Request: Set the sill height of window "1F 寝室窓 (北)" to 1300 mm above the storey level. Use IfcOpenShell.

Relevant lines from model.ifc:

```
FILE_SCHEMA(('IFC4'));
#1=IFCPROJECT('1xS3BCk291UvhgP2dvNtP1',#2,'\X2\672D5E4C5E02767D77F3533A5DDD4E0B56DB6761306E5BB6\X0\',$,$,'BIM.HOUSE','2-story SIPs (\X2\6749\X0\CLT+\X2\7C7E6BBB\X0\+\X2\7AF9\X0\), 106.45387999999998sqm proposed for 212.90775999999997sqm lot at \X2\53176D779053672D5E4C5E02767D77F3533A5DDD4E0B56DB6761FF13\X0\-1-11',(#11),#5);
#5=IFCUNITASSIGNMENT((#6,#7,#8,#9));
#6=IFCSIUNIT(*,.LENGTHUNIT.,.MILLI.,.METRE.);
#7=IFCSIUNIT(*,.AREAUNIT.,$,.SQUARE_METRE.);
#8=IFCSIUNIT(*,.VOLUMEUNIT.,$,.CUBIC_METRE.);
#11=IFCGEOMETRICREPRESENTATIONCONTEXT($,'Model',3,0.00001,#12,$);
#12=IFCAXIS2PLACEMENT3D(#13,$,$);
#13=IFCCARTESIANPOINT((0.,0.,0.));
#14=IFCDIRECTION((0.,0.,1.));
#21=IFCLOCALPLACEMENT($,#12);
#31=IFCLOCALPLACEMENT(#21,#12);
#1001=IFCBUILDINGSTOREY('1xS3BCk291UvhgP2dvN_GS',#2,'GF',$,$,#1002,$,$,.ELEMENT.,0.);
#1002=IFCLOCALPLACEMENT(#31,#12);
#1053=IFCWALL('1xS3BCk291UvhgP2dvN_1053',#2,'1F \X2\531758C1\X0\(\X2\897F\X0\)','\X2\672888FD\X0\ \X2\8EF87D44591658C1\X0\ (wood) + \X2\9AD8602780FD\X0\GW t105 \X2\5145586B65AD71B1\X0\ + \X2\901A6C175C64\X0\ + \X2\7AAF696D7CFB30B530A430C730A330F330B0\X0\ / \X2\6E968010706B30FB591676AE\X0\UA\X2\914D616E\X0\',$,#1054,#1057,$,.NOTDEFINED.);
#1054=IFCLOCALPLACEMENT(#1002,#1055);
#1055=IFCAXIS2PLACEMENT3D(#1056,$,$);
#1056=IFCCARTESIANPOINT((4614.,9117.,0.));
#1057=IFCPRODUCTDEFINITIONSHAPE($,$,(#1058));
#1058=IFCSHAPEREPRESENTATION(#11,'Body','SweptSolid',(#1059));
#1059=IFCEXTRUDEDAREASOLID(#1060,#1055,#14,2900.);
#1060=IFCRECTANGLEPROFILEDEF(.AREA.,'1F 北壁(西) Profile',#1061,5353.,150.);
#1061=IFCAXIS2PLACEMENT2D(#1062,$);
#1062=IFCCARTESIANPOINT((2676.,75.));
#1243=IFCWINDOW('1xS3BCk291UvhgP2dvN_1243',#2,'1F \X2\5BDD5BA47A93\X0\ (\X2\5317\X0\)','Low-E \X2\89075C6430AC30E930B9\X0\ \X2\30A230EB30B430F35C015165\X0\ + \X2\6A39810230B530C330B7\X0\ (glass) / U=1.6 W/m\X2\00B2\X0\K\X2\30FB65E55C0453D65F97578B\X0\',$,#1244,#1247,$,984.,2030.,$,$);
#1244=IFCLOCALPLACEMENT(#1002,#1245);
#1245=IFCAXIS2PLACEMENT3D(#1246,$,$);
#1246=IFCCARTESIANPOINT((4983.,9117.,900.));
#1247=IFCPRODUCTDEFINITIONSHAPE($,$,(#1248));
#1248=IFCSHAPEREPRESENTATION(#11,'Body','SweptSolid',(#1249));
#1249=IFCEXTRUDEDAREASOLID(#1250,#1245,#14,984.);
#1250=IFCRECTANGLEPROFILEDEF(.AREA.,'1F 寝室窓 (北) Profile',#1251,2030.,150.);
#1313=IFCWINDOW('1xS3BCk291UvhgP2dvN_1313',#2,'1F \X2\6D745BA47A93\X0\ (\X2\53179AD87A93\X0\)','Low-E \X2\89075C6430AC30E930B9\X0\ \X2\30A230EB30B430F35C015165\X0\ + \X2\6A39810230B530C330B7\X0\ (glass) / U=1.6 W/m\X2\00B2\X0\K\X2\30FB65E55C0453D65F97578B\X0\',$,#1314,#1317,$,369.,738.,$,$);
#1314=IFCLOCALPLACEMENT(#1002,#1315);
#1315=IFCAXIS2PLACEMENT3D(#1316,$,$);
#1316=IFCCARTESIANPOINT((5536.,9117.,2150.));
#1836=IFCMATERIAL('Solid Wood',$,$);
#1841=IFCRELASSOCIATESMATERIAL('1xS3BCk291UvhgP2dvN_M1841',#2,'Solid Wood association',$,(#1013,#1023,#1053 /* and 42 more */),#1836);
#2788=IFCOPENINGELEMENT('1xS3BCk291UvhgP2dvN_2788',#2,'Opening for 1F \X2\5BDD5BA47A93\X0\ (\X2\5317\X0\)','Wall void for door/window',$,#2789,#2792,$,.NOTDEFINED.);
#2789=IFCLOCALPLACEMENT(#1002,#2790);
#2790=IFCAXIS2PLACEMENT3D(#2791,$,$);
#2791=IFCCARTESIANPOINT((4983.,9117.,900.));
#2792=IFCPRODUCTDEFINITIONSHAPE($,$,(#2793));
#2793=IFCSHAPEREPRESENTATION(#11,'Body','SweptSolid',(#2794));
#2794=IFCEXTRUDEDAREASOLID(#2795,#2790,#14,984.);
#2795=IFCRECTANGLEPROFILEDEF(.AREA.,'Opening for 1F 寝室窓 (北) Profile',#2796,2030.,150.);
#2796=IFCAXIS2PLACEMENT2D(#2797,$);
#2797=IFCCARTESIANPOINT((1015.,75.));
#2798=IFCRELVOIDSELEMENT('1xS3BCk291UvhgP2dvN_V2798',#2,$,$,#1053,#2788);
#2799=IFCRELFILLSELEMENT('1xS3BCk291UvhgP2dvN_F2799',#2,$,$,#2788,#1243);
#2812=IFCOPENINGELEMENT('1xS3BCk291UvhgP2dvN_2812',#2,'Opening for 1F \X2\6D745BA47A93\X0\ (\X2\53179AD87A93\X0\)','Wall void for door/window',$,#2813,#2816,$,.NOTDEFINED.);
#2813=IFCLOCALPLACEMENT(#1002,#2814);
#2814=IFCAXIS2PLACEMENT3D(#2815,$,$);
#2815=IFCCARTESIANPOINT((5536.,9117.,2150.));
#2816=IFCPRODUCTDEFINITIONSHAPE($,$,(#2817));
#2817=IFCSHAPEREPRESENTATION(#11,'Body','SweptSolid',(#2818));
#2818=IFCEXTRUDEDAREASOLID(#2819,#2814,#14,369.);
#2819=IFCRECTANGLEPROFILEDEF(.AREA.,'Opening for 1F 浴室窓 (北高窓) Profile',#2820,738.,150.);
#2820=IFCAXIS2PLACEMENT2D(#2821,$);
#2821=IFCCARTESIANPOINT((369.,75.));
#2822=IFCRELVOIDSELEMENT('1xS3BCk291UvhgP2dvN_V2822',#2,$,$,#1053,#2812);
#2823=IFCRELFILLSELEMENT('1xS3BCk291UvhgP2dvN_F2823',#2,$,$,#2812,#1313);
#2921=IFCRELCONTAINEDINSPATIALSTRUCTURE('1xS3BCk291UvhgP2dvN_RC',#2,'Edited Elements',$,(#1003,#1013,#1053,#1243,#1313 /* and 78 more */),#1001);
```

```python
import numpy as np
import ifcopenshell
import ifcopenshell.api.geometry
import ifcopenshell.geom
import ifcopenshell.util.element
import ifcopenshell.util.placement
import ifcopenshell.util.shape
import ifcopenshell.util.unit

model = ifcopenshell.open("model.ifc")
unit_scale = ifcopenshell.util.unit.calculate_unit_scale(model)

window = model.by_guid("1xS3BCk291UvhgP2dvN_1243")
opening = window.FillsVoids[0].RelatingOpeningElement
storey = ifcopenshell.util.element.get_container(window, ifc_class="IfcBuildingStorey")
level = ifcopenshell.util.placement.get_local_placement(storey.ObjectPlacement)[2, 3]

# The opening's origin need not be at the sill, so measure its lowest point.
shape = ifcopenshell.geom.create_shape(ifcopenshell.geom.settings(), opening)
bottom = ifcopenshell.util.shape.get_shape_bottom_elevation(shape, shape.geometry) / unit_scale
dz = level + 1.3 / unit_scale - bottom

shift = np.array([0.0, 0.0, dz])
# The window is not placed relative to its opening, so move both.
for product in (opening, window):
    matrix = ifcopenshell.util.placement.get_local_placement(product.ObjectPlacement)
    matrix[:3, 3] += shift
    ifcopenshell.api.geometry.edit_object_placement(model, product=product, matrix=matrix, is_si=False)

print(f"moved by {dz * unit_scale:+.3f} m")

model.write("model-out.ifc")
```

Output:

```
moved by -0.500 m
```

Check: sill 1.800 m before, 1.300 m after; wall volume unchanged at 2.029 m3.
